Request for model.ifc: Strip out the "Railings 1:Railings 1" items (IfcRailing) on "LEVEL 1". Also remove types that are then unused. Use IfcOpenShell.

First a look at what the model holds.

```python
import ifcopenshell
import ifcopenshell.util.element

model = ifcopenshell.open("model.ifc")
print(model.schema)
storey = next(s for s in model.by_type("IfcBuildingStorey") if s.Name == "LEVEL 1")
railings = [e for e in ifcopenshell.util.element.get_decomposition(storey) if e.is_a("IfcRailing")]
seen = {}
for e in railings:
    element_type = ifcopenshell.util.element.get_type(e)
    name = element_type.Name if element_type not in (None, e) else None
    seen[name] = seen.get(name, 0) + 1
for name, count in sorted(seen.items(), key=str):
    print(count, "x", name)
```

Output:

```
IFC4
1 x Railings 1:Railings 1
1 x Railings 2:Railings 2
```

```python
import ifcopenshell
import ifcopenshell.api.root
import ifcopenshell.util.element

model = ifcopenshell.open("model.ifc")

storey = next(s for s in model.by_type("IfcBuildingStorey") if s.Name == "LEVEL 1")
railings = [e for e in ifcopenshell.util.element.get_decomposition(storey) if e.is_a("IfcRailing")]
targets = [e for e in railings if (t := ifcopenshell.util.element.get_type(e)) not in (None, e) and t.Name == "Railings 1:Railings 1"]
types = {ifcopenshell.util.element.get_type(e) for e in targets} - {None, *targets}

for e in targets:
    ifcopenshell.api.root.remove_product(model, product=e)
print(len(targets), "removed")

unused = [t for t in types if not ifcopenshell.util.element.get_types(t)]
for t in unused:
    ifcopenshell.api.root.remove_product(model, product=t)
print(len(unused), "unused types removed")

model.write("model_v2.ifc")
```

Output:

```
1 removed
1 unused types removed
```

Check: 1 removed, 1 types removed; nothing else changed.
